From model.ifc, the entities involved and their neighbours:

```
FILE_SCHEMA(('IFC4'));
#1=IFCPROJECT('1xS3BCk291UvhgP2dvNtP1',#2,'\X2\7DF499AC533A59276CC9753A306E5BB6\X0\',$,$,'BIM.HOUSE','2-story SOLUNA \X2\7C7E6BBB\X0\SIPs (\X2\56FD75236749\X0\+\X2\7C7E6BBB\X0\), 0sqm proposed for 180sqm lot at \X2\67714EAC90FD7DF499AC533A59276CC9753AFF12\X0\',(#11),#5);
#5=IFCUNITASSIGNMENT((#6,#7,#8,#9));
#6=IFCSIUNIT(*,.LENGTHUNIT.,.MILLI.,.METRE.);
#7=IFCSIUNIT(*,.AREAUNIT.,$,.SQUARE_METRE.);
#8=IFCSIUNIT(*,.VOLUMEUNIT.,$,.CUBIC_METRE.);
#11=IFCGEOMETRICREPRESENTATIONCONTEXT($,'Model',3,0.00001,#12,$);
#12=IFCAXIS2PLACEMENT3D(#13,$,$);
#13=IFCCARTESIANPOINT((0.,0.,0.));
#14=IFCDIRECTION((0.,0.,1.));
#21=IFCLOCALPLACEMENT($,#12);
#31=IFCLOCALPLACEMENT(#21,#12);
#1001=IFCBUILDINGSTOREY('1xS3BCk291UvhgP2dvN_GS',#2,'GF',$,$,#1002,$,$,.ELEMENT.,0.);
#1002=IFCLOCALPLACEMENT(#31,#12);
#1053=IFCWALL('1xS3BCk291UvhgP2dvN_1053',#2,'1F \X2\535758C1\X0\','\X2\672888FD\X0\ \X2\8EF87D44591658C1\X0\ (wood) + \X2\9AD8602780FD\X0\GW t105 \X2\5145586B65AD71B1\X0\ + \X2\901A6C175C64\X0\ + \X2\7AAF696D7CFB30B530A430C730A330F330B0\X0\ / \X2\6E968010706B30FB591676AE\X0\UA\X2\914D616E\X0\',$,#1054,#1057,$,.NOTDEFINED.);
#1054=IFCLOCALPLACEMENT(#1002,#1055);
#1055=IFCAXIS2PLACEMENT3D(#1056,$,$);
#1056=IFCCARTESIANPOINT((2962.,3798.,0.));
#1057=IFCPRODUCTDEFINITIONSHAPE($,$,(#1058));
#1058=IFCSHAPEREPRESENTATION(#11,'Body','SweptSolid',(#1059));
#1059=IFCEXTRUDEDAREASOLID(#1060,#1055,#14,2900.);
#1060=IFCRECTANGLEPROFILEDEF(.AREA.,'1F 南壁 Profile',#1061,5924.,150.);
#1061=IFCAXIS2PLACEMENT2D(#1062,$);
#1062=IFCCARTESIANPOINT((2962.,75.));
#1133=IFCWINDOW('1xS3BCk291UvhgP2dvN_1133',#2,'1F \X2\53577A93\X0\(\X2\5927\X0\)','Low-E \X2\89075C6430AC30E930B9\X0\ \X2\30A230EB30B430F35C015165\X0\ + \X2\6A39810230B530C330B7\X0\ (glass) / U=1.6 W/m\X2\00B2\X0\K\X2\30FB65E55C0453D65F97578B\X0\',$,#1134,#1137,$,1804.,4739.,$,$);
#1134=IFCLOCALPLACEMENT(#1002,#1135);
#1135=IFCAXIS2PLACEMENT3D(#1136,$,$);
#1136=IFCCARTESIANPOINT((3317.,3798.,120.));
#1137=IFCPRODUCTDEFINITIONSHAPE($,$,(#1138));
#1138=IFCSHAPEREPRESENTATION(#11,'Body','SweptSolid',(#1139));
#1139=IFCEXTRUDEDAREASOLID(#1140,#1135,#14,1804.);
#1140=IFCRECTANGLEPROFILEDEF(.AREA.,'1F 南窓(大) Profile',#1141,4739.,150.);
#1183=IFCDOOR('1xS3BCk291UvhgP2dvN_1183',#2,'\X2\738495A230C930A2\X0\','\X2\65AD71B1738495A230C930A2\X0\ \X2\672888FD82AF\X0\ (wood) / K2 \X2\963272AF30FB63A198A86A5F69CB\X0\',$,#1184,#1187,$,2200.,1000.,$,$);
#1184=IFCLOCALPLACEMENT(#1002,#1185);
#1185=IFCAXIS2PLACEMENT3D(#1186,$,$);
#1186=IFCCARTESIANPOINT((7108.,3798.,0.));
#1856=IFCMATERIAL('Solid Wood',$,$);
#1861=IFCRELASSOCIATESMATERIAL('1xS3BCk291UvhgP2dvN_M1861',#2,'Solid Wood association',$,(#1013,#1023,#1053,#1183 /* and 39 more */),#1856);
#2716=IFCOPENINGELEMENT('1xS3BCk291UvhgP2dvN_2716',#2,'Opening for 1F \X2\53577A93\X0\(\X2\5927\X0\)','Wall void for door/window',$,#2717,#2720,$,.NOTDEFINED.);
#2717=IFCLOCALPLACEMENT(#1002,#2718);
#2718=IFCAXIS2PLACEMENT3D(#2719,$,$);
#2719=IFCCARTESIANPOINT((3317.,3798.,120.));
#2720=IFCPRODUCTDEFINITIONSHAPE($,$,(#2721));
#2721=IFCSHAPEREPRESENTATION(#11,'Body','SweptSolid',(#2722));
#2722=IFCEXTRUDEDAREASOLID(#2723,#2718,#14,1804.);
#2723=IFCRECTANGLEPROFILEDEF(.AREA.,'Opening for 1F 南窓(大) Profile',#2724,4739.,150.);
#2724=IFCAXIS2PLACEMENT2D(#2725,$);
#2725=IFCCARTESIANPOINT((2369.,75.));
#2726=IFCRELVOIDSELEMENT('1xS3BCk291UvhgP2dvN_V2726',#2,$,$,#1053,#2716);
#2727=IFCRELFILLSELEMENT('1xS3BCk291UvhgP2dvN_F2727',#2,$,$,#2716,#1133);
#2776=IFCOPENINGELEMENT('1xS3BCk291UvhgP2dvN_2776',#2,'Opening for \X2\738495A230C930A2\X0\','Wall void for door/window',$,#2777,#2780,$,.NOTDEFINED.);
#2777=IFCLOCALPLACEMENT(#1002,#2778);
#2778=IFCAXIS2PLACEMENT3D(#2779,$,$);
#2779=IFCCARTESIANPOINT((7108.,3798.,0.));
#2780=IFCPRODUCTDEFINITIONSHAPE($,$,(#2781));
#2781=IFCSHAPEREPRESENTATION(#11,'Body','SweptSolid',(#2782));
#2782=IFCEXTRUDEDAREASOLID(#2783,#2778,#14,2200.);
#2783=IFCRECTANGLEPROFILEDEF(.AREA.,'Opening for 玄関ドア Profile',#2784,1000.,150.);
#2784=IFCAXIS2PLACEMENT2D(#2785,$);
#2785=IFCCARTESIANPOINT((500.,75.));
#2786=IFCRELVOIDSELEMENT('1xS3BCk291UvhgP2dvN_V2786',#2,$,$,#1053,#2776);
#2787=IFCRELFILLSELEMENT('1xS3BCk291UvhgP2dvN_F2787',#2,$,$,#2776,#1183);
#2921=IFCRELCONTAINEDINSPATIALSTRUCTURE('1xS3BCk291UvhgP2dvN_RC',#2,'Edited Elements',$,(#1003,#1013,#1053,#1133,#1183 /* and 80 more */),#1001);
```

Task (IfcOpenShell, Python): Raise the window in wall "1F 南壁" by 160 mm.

```python
import numpy as np
import ifcopenshell
import ifcopenshell.api.geometry
import ifcopenshell.util.placement
import ifcopenshell.util.unit

model = ifcopenshell.open("model.ifc")
unit_scale = ifcopenshell.util.unit.calculate_unit_scale(model)

window = model.by_guid("1xS3BCk291UvhgP2dvN_1133")
opening = window.FillsVoids[0].RelatingOpeningElement
dz = 0.16 / unit_scale

shift = np.array([0.0, 0.0, dz])
# The window is not placed relative to its opening, so move both.
for product in (opening, window):
    matrix = ifcopenshell.util.placement.get_local_placement(product.ObjectPlacement)
    matrix[:3, 3] += shift
    ifcopenshell.api.geometry.edit_object_placement(model, product=product, matrix=matrix, is_si=False)

print(f"moved by {dz * unit_scale:+.3f} m")

model.write("model_rev.ifc")
```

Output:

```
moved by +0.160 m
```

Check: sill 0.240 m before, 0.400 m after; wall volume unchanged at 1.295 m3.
